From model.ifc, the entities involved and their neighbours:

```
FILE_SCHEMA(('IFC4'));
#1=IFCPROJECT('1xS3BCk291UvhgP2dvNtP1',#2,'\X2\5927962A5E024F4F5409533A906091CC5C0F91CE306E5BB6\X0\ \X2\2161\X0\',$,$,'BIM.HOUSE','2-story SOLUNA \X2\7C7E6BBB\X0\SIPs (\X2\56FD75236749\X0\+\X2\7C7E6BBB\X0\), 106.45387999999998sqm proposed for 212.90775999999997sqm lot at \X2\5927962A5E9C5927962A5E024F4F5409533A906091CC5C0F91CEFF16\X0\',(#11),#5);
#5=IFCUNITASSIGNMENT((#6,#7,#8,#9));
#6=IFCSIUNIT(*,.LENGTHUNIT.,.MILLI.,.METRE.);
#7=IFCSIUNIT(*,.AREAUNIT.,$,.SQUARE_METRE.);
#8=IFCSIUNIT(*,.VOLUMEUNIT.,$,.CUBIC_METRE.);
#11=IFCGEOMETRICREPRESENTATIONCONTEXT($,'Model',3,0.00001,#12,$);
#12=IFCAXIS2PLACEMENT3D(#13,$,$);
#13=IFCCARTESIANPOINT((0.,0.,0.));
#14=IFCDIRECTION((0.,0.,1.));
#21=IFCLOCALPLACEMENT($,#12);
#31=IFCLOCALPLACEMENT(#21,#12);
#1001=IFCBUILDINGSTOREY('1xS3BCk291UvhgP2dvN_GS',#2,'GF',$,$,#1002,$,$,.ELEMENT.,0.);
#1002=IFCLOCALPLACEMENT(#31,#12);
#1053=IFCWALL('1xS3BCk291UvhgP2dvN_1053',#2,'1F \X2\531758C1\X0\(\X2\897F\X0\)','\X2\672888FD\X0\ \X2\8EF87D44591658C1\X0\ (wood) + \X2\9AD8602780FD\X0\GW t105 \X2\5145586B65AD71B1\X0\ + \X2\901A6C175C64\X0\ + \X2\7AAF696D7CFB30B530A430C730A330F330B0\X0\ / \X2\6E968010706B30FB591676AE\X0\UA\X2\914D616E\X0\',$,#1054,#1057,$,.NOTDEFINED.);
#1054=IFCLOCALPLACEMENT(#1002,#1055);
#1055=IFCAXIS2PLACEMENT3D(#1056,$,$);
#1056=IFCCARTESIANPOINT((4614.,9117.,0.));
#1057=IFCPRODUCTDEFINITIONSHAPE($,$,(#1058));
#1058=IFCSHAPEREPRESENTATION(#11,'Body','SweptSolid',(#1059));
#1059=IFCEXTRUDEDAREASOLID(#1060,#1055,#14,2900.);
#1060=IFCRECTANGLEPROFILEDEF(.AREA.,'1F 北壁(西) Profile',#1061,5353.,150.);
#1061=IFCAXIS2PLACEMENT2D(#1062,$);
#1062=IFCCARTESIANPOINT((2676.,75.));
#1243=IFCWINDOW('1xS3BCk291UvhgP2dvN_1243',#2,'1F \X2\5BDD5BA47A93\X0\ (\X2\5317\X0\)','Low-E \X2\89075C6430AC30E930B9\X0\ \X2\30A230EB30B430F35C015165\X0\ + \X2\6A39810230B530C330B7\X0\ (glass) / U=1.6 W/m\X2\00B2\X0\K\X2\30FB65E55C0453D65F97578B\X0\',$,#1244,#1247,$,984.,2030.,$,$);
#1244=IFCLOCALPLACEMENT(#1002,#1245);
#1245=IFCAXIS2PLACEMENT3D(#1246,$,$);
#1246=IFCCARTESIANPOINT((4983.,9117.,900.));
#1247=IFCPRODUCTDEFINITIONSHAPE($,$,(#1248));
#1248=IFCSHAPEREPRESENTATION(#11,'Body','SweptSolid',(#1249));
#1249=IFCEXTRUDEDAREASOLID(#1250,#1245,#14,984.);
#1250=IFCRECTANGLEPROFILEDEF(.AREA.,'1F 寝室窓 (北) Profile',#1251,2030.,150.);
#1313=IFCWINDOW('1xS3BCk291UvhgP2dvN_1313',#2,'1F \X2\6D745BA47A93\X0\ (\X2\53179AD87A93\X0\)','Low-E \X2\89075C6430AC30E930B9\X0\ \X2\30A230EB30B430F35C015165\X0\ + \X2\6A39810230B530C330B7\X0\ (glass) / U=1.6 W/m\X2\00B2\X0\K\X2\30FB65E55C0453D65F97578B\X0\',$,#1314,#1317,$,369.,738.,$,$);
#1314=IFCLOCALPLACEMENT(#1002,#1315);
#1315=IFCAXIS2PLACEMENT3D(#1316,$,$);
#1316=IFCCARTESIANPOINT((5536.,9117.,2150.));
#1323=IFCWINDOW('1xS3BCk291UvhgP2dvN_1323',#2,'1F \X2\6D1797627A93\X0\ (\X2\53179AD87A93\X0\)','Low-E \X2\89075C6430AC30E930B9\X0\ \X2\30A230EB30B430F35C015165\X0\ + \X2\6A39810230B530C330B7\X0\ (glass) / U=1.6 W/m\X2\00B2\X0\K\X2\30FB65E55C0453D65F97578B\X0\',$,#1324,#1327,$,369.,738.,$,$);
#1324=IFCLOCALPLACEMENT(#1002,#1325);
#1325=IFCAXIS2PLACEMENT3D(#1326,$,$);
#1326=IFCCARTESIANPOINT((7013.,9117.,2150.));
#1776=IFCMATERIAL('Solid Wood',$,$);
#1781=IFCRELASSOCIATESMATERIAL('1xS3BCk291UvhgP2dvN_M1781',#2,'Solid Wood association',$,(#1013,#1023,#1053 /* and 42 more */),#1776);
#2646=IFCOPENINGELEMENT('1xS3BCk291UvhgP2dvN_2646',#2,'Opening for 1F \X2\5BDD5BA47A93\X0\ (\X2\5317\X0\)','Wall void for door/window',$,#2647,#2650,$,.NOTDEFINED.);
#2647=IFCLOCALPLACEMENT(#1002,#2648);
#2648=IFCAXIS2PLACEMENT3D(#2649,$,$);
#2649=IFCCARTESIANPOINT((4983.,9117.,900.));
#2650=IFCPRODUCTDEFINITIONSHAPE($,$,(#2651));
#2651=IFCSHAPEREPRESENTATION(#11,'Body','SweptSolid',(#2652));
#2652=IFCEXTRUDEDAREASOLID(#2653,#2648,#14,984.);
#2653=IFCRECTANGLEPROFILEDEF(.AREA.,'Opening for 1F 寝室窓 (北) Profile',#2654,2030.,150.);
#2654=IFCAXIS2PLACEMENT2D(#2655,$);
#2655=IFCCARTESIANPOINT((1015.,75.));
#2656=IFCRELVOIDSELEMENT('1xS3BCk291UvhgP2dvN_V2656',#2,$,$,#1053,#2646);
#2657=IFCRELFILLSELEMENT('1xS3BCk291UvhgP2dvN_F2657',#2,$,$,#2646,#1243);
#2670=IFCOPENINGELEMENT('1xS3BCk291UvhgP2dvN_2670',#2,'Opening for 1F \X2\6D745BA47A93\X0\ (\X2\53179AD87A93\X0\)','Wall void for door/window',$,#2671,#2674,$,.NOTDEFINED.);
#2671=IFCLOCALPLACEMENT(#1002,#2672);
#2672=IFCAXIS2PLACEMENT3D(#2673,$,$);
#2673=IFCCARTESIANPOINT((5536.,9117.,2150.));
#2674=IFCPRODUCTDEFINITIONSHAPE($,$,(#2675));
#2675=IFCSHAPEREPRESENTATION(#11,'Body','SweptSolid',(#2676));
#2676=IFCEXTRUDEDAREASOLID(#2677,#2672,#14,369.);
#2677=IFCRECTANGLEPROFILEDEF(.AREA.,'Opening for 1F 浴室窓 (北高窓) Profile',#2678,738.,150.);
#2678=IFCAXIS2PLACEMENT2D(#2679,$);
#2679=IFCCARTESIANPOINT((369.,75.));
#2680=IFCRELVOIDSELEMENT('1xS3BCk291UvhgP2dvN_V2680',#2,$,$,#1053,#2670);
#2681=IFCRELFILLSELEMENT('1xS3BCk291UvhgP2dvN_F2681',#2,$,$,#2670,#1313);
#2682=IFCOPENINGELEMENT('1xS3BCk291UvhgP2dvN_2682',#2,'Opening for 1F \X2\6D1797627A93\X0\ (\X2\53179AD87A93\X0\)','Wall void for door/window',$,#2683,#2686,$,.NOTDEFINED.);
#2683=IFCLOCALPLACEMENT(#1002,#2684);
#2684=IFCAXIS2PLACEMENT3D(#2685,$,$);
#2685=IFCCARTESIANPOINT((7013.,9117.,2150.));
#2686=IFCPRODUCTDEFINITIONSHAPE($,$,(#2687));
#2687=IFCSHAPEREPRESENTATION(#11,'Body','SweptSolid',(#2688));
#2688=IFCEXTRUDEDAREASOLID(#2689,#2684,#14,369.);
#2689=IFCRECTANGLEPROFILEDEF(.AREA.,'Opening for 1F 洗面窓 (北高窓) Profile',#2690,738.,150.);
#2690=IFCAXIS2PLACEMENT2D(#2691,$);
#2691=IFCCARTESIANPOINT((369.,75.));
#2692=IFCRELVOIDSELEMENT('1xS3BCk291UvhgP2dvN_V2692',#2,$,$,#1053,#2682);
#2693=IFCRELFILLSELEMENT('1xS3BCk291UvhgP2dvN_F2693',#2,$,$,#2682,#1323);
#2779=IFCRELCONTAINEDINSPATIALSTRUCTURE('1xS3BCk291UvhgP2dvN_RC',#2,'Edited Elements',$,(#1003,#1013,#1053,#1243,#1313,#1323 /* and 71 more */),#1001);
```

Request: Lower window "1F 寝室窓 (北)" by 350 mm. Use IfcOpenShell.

```python
import numpy as np
import ifcopenshell
import ifcopenshell.api.geometry
import ifcopenshell.util.placement
import ifcopenshell.util.unit

model = ifcopenshell.open("model.ifc")
unit_scale = ifcopenshell.util.unit.calculate_unit_scale(model)

window = model.by_id(1243)
opening = window.FillsVoids[0].RelatingOpeningElement
dz = -350.0

shift = np.array([0.0, 0.0, dz])
# The window is not placed relative to its opening, so move both.
for product in (opening, window):
    matrix = ifcopenshell.util.placement.get_local_placement(product.ObjectPlacement)
    matrix[:3, 3] += shift
    ifcopenshell.api.geometry.edit_object_placement(model, product=product, matrix=matrix, is_si=False)

print(f"moved by {dz * unit_scale:+.3f} m")

model.write("model_rev.ifc")
```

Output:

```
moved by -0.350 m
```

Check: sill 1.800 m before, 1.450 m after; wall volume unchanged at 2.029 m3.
